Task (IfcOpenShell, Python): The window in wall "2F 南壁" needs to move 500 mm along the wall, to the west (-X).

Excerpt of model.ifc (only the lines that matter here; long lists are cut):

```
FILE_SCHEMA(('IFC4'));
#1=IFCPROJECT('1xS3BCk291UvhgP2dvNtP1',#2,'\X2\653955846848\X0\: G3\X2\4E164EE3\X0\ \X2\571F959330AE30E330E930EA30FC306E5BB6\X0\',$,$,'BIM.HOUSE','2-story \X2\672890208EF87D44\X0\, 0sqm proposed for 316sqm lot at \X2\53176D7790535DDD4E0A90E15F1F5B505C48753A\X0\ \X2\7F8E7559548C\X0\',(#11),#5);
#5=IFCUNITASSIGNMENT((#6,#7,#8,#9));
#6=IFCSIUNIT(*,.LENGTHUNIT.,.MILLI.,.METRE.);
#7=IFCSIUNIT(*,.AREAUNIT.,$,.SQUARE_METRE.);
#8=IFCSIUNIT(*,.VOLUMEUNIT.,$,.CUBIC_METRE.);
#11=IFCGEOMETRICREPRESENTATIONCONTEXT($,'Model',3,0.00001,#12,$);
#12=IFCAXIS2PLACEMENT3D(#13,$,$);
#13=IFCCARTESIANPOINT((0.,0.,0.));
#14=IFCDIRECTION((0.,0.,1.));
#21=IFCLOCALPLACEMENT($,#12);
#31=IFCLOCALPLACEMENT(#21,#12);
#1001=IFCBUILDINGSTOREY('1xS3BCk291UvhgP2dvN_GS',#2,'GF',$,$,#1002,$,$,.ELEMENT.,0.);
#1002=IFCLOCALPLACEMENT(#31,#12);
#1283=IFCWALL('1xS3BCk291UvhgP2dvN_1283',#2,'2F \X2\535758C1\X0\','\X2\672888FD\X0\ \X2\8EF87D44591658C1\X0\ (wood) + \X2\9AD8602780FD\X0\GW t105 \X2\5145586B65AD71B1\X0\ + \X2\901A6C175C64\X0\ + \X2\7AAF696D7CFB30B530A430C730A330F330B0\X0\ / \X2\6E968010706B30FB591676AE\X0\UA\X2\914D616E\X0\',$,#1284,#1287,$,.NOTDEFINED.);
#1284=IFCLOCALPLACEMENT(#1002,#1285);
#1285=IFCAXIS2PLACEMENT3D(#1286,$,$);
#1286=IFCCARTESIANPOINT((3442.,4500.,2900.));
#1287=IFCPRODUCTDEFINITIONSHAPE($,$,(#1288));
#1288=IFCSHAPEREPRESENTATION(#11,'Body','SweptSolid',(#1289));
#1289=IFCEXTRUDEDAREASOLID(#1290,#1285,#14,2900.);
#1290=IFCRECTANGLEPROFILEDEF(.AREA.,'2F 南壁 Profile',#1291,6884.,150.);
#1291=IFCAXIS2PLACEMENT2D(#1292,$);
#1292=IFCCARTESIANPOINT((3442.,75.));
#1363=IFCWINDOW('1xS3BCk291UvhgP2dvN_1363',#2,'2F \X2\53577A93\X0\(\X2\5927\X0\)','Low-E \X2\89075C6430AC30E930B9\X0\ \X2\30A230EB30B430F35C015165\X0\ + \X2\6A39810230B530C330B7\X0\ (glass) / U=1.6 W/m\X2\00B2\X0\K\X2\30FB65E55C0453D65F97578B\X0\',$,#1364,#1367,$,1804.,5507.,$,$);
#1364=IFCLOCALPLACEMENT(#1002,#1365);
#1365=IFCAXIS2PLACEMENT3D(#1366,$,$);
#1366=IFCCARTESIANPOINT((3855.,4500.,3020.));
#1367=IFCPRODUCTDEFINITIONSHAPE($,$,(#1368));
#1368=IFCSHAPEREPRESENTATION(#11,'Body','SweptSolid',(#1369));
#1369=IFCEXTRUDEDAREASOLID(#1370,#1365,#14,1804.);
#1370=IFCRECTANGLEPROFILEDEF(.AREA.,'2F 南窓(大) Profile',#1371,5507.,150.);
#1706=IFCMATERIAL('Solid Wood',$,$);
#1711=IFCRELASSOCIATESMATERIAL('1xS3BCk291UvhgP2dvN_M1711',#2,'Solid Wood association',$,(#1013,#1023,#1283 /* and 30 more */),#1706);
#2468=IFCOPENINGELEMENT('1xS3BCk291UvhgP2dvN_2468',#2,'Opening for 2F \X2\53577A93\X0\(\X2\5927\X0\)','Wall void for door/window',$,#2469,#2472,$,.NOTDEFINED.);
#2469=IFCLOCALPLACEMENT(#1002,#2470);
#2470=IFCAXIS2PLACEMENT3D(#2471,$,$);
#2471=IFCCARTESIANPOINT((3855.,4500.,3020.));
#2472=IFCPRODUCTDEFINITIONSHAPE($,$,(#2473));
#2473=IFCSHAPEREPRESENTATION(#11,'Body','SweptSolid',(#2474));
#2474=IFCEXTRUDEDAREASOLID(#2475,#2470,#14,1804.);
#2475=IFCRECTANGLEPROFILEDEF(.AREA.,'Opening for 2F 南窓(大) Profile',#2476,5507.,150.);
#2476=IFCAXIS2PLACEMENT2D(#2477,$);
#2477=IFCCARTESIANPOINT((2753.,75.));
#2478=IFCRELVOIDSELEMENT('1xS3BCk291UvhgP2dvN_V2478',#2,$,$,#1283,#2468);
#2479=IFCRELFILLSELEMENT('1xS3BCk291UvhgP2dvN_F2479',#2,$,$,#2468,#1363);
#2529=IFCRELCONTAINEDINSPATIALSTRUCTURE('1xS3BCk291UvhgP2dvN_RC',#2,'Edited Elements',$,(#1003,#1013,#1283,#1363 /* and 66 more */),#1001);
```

```python
import ifcopenshell
import ifcopenshell.api.geometry
import ifcopenshell.util.placement

model = ifcopenshell.open("model.ifc")

window = model.by_guid("1xS3BCk291UvhgP2dvN_1363")
opening = window.FillsVoids[0].RelatingOpeningElement
wall = opening.VoidsElements[0].RelatingBuildingElement

wall_matrix = ifcopenshell.util.placement.get_local_placement(wall.ObjectPlacement)
shift = wall_matrix[:3, 0] * -500.0
before = ifcopenshell.util.placement.get_local_placement(window.ObjectPlacement)[:3, 3].copy()

# The window is not placed relative to its opening, so move both.
for product in (opening, window):
    matrix = ifcopenshell.util.placement.get_local_placement(product.ObjectPlacement)
    matrix[:3, 3] += shift
    ifcopenshell.api.geometry.edit_object_placement(model, product=product, matrix=matrix, is_si=False)

after = ifcopenshell.util.placement.get_local_placement(window.ObjectPlacement)[:3, 3]
print("window moved by", (after - before).round(3) + 0.0)

model.write("model_edited.ifc")
```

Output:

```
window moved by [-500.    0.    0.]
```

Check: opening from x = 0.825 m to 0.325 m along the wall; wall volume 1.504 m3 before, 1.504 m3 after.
